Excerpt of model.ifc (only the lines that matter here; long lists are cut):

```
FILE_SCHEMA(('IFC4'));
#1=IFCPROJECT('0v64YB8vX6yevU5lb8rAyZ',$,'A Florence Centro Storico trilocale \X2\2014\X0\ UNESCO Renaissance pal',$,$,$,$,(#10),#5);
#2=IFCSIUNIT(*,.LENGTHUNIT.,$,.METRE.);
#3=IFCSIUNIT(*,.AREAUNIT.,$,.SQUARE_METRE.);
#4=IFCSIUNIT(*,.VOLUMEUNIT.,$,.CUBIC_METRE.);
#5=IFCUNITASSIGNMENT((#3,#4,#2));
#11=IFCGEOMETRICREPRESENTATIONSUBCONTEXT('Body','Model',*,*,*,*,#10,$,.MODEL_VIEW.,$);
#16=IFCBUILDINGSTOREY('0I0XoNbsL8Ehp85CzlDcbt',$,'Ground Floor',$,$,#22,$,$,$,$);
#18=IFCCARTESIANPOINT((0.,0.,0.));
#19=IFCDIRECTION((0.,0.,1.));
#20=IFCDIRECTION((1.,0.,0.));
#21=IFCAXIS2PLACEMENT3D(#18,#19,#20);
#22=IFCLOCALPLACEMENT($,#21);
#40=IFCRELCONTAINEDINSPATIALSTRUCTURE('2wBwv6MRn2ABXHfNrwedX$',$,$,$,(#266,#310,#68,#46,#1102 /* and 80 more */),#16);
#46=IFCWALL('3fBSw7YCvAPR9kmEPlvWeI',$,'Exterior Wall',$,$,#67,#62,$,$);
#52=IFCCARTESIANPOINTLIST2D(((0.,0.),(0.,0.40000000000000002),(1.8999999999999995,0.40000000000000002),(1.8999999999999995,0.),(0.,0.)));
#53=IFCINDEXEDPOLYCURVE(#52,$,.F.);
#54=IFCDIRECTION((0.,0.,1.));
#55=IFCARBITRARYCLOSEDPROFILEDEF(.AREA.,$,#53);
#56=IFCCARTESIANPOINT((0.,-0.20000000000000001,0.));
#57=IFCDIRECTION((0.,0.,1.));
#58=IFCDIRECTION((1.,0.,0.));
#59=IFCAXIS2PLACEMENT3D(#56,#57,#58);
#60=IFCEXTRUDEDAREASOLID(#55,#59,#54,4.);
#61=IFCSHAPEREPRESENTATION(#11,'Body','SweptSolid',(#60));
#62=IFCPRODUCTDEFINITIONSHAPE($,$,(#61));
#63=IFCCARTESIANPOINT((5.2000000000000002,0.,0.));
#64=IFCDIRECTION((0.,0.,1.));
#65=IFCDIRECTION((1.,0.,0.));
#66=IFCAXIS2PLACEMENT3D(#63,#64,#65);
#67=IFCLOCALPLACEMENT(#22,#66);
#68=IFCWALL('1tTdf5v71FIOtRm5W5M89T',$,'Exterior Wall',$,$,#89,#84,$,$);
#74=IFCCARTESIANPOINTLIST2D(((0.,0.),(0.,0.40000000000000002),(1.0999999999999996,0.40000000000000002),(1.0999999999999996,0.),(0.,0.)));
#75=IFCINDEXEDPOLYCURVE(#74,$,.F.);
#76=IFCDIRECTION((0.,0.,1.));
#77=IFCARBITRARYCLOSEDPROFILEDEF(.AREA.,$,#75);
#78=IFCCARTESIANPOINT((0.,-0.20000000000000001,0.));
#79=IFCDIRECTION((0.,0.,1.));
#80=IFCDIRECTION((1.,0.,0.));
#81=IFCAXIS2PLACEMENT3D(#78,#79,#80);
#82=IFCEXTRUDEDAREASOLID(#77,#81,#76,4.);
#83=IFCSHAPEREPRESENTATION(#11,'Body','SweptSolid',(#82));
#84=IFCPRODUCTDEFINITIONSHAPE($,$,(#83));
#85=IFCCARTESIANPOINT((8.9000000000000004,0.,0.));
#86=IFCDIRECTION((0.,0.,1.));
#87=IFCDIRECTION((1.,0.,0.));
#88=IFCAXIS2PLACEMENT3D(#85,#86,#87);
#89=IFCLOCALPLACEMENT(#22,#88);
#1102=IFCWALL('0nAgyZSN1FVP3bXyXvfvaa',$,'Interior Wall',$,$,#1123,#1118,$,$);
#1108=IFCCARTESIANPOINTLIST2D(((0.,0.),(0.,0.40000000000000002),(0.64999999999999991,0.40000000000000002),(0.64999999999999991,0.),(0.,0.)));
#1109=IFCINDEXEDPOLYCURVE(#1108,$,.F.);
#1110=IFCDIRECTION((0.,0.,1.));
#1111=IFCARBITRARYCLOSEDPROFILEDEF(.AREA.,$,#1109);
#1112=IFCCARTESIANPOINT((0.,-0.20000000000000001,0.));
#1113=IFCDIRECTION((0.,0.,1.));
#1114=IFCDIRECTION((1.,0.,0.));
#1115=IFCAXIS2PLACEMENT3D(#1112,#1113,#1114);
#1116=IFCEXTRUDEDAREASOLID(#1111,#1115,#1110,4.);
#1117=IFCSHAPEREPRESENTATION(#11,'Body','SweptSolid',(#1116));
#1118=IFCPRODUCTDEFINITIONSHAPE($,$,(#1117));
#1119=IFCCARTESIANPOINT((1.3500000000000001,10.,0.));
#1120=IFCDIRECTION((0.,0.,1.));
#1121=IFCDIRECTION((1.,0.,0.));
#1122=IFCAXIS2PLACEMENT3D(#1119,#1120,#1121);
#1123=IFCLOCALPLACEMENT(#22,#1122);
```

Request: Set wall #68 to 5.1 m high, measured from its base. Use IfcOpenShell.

```python
import ifcopenshell
import ifcopenshell.geom
import ifcopenshell.util.representation
import ifcopenshell.util.shape
import ifcopenshell.util.unit

model = ifcopenshell.open("model.ifc")
unit_scale = ifcopenshell.util.unit.calculate_unit_scale(model)
settings = ifcopenshell.geom.settings()


def volume(element):
    """Net volume in cubic metres, openings subtracted."""
    shape = ifcopenshell.geom.create_shape(settings, element)
    return ifcopenshell.util.shape.get_volume(shape.geometry)


wall = model.by_guid("1tTdf5v71FIOtRm5W5M89T")
before = volume(wall)

body = ifcopenshell.util.representation.get_representation(wall, "Model", "Body")
solid = body.Items[0]
old_height = solid.Depth
solid.Depth = 5.1 / unit_scale
after = volume(wall)

print(f"height {old_height:g} -> {solid.Depth:g}, volume {before:.3f} -> {after:.3f} m3")

model.write("model_edited.ifc")
```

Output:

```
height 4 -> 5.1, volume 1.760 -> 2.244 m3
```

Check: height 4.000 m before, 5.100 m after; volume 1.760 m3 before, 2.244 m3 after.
